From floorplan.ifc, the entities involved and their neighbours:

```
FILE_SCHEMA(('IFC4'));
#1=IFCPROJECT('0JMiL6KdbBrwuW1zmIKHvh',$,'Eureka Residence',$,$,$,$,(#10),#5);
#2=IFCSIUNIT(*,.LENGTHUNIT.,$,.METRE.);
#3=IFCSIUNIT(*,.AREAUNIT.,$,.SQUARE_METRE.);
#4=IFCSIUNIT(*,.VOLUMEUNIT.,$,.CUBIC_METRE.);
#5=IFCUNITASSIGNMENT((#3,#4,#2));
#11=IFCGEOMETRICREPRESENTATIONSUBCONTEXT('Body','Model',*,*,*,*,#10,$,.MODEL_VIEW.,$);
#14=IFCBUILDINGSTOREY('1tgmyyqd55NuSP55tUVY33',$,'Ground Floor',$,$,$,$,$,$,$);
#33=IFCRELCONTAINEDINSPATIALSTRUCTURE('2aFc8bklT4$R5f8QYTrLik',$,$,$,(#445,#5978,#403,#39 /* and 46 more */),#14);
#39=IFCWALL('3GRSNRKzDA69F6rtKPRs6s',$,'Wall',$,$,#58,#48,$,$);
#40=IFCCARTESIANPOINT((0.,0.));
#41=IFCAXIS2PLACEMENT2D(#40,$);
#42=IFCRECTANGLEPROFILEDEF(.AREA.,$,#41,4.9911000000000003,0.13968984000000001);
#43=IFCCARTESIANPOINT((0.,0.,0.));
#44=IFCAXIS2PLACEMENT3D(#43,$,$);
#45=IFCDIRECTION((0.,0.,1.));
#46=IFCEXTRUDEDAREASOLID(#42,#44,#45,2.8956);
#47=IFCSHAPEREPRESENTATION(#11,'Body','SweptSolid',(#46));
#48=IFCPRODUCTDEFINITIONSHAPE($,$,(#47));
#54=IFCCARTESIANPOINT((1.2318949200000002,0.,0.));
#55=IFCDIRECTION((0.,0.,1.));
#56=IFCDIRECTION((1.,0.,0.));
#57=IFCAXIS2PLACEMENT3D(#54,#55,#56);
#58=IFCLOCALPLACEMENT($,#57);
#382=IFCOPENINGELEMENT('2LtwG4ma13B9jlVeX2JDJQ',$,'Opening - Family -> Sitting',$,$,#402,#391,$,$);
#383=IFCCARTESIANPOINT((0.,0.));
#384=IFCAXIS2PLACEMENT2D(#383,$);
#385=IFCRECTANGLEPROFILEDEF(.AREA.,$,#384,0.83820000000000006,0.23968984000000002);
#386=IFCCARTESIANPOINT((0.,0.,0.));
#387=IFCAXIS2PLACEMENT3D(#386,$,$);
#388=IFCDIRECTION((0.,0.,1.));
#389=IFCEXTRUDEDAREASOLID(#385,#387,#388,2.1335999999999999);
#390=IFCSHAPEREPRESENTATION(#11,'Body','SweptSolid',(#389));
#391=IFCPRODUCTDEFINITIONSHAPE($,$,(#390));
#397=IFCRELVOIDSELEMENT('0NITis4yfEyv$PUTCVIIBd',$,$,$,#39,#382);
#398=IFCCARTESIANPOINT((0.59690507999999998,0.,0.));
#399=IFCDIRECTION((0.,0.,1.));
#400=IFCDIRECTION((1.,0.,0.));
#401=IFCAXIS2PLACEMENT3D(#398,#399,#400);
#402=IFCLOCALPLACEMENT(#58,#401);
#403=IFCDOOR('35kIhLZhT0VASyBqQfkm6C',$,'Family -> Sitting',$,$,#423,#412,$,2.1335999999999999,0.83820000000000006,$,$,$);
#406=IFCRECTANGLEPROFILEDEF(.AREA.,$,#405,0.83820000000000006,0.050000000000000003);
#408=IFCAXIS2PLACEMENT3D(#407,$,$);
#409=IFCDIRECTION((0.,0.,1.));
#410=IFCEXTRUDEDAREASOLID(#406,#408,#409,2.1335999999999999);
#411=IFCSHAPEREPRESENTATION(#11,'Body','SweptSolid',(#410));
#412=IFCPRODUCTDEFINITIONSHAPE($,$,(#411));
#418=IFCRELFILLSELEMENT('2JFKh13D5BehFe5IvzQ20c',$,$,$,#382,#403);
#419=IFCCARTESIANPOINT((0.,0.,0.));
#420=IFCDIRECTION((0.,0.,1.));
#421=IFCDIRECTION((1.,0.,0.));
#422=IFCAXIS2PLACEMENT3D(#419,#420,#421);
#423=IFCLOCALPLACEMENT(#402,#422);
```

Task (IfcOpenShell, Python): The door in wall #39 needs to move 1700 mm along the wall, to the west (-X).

```python
import ifcopenshell
import ifcopenshell.api.geometry
import ifcopenshell.util.placement
import ifcopenshell.util.unit

model = ifcopenshell.open("floorplan.ifc")
unit_scale = ifcopenshell.util.unit.calculate_unit_scale(model)

door = model.by_guid("35kIhLZhT0VASyBqQfkm6C")
opening = door.FillsVoids[0].RelatingOpeningElement
wall = opening.VoidsElements[0].RelatingBuildingElement

wall_matrix = ifcopenshell.util.placement.get_local_placement(wall.ObjectPlacement)
shift = wall_matrix[:3, 0] * -1.7 / unit_scale
before = ifcopenshell.util.placement.get_local_placement(door.ObjectPlacement)[:3, 3].copy()

# The door is placed relative to its opening, so it follows when the opening moves.
matrix = ifcopenshell.util.placement.get_local_placement(opening.ObjectPlacement)
matrix[:3, 3] += shift
ifcopenshell.api.geometry.edit_object_placement(
    model, product=opening, matrix=matrix, is_si=False, should_transform_children=True
)

after = ifcopenshell.util.placement.get_local_placement(door.ObjectPlacement)[:3, 3]
print("door moved by", (after - before).round(3) + 0.0)

model.write("floorplan-out.ifc")
```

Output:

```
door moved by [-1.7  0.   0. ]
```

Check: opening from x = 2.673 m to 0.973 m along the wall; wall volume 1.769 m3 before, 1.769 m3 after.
